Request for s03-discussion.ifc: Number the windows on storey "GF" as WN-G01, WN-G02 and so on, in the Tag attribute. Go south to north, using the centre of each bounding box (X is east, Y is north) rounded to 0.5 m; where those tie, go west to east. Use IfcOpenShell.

First a look at what the model holds.

```python
import ifcopenshell
import ifcopenshell.util.element
import ifcopenshell.util.placement

model = ifcopenshell.open("s03-discussion.ifc")
print(model.schema)
storey = next(s for s in model.by_type("IfcBuildingStorey") if s.Name == "GF")
windows = [e for e in ifcopenshell.util.element.get_decomposition(storey) if e.is_a("IfcWindow")]
for e in sorted(windows, key=lambda e: e.id()):
    origin = ifcopenshell.util.placement.get_local_placement(e.ObjectPlacement)[:3, 3]
    print(e.id(), e.Tag, e.Name, origin.round(2) + 0.0, sep=" | ")
```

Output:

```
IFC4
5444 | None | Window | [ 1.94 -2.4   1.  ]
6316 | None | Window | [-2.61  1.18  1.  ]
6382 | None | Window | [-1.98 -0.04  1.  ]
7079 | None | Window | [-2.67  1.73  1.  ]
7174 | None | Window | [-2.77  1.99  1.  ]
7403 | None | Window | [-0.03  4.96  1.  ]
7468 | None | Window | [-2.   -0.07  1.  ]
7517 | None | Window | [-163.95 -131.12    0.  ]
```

```python
import ifcopenshell
import ifcopenshell.geom
import ifcopenshell.util.element
import ifcopenshell.util.shape

model = ifcopenshell.open("s03-discussion.ifc")
settings = ifcopenshell.geom.settings()
settings.set("use-world-coords", True)


def centre(element):
    shape = ifcopenshell.geom.create_shape(settings, element)
    return ifcopenshell.util.shape.get_bbox_centroid(shape.geometry)


storey = next(s for s in model.by_type("IfcBuildingStorey") if s.Name == "GF")
windows = [e for e in ifcopenshell.util.element.get_decomposition(storey) if e.is_a("IfcWindow")]

# Insertion points can sit at a corner or the storey origin, so sort by the geometry (in metres).
centres = {e: centre(e) for e in windows}
windows.sort(key=lambda e: (round(centres[e][1] / 0.5), centres[e][0]))

for i, e in enumerate(windows, start=1):
    number = f"WN-G{i:02d}"
    e.Tag = number
    print(e.id(), number)

model.write("s03-discussion-out.ifc")
```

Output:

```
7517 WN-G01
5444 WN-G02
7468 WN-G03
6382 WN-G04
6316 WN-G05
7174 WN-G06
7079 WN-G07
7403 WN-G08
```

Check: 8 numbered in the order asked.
